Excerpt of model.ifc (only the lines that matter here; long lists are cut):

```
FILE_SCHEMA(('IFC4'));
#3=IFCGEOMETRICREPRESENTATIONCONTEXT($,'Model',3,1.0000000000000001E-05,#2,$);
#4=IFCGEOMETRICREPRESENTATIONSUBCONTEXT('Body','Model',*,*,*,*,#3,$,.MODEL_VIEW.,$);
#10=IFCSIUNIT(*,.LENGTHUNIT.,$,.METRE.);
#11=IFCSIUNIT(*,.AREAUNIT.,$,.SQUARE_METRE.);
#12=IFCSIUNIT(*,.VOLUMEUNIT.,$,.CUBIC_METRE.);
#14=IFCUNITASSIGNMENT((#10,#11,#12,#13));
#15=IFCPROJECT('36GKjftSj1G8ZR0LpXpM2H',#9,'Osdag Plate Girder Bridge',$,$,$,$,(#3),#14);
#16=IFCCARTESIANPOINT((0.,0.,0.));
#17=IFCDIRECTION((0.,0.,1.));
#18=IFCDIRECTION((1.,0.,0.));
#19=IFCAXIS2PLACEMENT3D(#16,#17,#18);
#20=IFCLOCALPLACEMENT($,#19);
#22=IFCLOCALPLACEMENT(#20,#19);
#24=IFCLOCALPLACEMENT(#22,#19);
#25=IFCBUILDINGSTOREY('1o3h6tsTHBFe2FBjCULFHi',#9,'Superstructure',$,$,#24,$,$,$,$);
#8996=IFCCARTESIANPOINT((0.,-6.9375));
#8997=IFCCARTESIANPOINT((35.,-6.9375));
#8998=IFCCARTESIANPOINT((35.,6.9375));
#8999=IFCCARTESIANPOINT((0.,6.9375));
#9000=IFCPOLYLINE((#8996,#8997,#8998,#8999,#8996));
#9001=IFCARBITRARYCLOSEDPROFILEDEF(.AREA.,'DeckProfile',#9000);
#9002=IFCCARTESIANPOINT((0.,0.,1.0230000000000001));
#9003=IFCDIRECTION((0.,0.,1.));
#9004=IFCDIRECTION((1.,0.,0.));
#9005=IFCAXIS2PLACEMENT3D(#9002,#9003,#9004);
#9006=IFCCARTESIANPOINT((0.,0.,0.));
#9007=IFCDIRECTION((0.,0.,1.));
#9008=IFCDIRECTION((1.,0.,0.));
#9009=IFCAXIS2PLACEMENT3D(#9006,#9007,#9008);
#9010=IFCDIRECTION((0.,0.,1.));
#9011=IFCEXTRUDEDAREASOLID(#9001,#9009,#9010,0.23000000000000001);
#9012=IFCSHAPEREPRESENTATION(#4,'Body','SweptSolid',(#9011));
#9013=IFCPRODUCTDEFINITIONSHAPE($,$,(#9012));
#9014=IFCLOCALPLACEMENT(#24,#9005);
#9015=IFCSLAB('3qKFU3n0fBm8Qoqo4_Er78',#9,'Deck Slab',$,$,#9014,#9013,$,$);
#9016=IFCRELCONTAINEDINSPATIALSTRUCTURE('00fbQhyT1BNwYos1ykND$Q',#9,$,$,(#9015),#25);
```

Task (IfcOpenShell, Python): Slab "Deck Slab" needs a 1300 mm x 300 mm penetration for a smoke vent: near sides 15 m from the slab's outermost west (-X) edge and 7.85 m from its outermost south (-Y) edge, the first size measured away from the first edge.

```python
import numpy as np
import ifcopenshell
import ifcopenshell.api.feature
import ifcopenshell.api.geometry
import ifcopenshell.api.root
import ifcopenshell.geom
import ifcopenshell.util.placement
import ifcopenshell.util.representation
import ifcopenshell.util.shape
import ifcopenshell.util.unit

model = ifcopenshell.open("model.ifc")
unit_scale = ifcopenshell.util.unit.calculate_unit_scale(model)
settings = ifcopenshell.geom.settings()


def volume(element):
    """Net volume in cubic metres, openings subtracted."""
    shape = ifcopenshell.geom.create_shape(settings, element)
    return ifcopenshell.util.shape.get_volume(shape.geometry)


slab = model.by_guid("3qKFU3n0fBm8Qoqo4_Er78")
before = volume(slab)

# Extent in the slab's own axes, in metres. The edges named are its -X and -Y sides.
slab_shape = ifcopenshell.geom.create_shape(settings, slab)
vertices = ifcopenshell.util.shape.get_vertices(slab_shape.geometry)
x_min, y_min, bottom = vertices.min(axis=0)
top = vertices[:, 2].max()

opening = ifcopenshell.api.root.create_entity(model, ifc_class="IfcOpeningElement", name="Smoke vent opening", predefined_type="OPENING")
context = ifcopenshell.util.representation.get_context(model, "Model", "Body", "MODEL_VIEW")
width, depth = 1.3, 0.3
outline = [(0.0, 0.0), (width, 0.0), (width, depth), (0.0, depth), (0.0, 0.0)]
# Overshoot both faces by 50 mm so the cut is clean.
shape = ifcopenshell.api.geometry.add_slab_representation(
    model, context=context, depth=top - bottom + 0.1, polyline=outline
)
ifcopenshell.api.geometry.assign_representation(model, product=opening, representation=shape)

matrix = ifcopenshell.util.placement.get_local_placement(slab.ObjectPlacement)
matrix[:, 3] = matrix @ np.append(np.array([x_min + 15, y_min + 7.85, bottom - 0.05]) / unit_scale, 1.0)
ifcopenshell.api.geometry.edit_object_placement(model, product=opening, matrix=matrix, is_si=False)
ifcopenshell.api.feature.add_feature(model, feature=opening, element=slab)

after = volume(slab)

print(f"slab volume {before:.3f} -> {after:.3f} m3")

model.write("model-out.ifc")
```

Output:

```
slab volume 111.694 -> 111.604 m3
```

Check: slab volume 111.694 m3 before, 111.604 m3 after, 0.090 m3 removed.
